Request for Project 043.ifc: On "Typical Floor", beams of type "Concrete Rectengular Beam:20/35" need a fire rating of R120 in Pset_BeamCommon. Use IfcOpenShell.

First a look at what the model holds.

```python
import ifcopenshell
import ifcopenshell.util.element

model = ifcopenshell.open("Project 043.ifc")
print(model.schema)
storey = next(s for s in model.by_type("IfcBuildingStorey") if s.Name == "Typical Floor")
beams = [e for e in ifcopenshell.util.element.get_decomposition(storey) if e.is_a("IfcBeam")]
seen = {}
for e in beams:
    element_type = ifcopenshell.util.element.get_type(e)
    key = (element_type.Name if element_type != e and element_type else None, ifcopenshell.util.element.get_pset(e, "Pset_BeamCommon", "FireRating"))
    seen[key] = seen.get(key, 0) + 1
for (name, value), count in sorted(seen.items(), key=str):
    print(count, "x", name, "|", value)
```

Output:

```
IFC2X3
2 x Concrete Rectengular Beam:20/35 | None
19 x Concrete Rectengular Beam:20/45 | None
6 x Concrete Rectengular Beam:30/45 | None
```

```python
import ifcopenshell
import ifcopenshell.api.pset
import ifcopenshell.util.element

model = ifcopenshell.open("Project 043.ifc")

storey = next(s for s in model.by_type("IfcBuildingStorey") if s.Name == "Typical Floor")
beams = [e for e in ifcopenshell.util.element.get_decomposition(storey) if e.is_a("IfcBeam")]

count = 0
for e in beams:
    element_type = ifcopenshell.util.element.get_type(e)
    if element_type in (None, e) or element_type.Name != "Concrete Rectengular Beam:20/35":
        continue
    # add_pset returns the element's existing set when there is one.
    pset = ifcopenshell.api.pset.add_pset(model, product=e, name="Pset_BeamCommon")
    ifcopenshell.api.pset.edit_pset(model, pset=pset, properties={"FireRating": "R120"})
    count += 1

print(count, "beams updated")

model.write("Project 043_rev.ifc")
```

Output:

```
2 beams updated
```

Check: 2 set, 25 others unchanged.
